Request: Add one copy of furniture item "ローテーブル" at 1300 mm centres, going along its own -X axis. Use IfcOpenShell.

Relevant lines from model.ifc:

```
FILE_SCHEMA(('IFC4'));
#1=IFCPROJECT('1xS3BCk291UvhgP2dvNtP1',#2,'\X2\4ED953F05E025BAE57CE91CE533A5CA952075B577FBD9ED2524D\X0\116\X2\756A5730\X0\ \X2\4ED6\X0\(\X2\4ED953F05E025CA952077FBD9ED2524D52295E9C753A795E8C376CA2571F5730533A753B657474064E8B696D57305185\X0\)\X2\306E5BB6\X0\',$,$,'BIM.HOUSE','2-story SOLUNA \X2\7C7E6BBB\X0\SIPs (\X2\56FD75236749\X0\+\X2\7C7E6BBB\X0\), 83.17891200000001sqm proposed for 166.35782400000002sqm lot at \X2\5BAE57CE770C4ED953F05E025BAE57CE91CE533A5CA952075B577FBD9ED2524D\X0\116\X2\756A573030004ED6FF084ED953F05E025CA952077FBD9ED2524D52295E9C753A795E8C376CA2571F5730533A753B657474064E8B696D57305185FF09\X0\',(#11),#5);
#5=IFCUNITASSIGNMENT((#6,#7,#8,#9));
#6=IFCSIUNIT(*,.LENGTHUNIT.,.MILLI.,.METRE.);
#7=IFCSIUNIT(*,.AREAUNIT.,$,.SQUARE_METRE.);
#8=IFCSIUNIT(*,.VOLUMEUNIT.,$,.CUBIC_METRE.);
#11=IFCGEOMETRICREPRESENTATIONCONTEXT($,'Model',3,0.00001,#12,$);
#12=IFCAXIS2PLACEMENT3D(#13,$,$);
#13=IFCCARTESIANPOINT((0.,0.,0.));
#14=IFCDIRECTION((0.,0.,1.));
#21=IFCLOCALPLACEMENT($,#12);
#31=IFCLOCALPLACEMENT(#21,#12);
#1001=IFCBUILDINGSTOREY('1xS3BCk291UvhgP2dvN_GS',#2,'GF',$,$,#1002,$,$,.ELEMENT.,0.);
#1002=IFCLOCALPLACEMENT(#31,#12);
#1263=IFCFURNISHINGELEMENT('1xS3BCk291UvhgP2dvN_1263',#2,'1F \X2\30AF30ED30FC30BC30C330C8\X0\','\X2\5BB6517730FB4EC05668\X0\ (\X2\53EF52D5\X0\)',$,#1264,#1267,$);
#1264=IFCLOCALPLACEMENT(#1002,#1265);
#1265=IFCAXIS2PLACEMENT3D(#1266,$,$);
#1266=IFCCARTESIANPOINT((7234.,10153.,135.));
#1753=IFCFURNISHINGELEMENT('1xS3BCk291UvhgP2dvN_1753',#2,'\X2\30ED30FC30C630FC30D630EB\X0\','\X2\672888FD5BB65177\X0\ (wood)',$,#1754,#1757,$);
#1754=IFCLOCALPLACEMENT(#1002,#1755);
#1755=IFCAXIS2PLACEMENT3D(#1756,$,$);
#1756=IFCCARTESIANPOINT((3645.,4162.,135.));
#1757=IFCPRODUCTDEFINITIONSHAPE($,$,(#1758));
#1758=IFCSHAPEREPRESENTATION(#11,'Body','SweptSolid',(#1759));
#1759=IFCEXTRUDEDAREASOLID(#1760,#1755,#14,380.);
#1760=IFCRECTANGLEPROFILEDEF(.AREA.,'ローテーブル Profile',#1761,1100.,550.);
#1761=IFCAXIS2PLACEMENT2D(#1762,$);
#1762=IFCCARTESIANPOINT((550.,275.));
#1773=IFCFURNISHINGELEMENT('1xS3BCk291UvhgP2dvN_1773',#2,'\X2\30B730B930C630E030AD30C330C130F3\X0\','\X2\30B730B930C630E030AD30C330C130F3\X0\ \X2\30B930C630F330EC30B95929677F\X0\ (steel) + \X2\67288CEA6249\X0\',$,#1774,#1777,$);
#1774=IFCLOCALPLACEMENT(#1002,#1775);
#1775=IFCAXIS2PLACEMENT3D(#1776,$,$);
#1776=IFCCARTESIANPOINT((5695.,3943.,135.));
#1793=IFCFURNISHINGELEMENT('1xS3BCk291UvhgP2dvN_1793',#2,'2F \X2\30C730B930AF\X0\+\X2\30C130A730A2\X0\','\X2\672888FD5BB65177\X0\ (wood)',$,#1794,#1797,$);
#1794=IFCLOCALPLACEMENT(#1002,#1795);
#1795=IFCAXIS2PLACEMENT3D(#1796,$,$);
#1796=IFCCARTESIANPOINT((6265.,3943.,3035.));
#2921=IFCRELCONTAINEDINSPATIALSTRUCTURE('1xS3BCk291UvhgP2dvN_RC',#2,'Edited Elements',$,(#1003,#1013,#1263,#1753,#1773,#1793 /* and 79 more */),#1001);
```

```python
import ifcopenshell
import ifcopenshell.api.geometry
import ifcopenshell.api.root
import ifcopenshell.util.element
import ifcopenshell.util.placement
import ifcopenshell.util.unit

model = ifcopenshell.open("model.ifc")
unit_scale = ifcopenshell.util.unit.calculate_unit_scale(model)


def reuse_history(source, copy):
    """copy_class also copies each property set's owner history, people and application; keep the originals."""
    for rel in copy.IsDefinedBy:
        if rel.is_a("IfcRelDefinesByProperties") and (history := rel.RelatingPropertyDefinition.OwnerHistory):
            rel.RelatingPropertyDefinition.OwnerHistory = source.OwnerHistory
            ifcopenshell.util.element.remove_deep2(model, history)


source = model.by_guid("1xS3BCk291UvhgP2dvN_1753")
base = ifcopenshell.util.placement.get_local_placement(source.ObjectPlacement)
step = -base[:3, 0] * 1.3 / unit_scale

for i in range(1, 2):
    copy = ifcopenshell.api.root.copy_class(model, product=source)
    copy.Representation = ifcopenshell.util.element.copy_deep(
        model, source.Representation, exclude=["IfcGeometricRepresentationContext", "IfcRepresentationMap"]
    )
    reuse_history(source, copy)
    matrix = base.copy()
    matrix[:3, 3] += i * step
    print("added at", matrix[:3, 3].round(3) + 0.0)
    ifcopenshell.api.geometry.edit_object_placement(model, product=copy, matrix=matrix, is_si=False)

model.write("model_rev.ifc")
```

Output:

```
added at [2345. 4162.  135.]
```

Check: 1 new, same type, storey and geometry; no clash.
